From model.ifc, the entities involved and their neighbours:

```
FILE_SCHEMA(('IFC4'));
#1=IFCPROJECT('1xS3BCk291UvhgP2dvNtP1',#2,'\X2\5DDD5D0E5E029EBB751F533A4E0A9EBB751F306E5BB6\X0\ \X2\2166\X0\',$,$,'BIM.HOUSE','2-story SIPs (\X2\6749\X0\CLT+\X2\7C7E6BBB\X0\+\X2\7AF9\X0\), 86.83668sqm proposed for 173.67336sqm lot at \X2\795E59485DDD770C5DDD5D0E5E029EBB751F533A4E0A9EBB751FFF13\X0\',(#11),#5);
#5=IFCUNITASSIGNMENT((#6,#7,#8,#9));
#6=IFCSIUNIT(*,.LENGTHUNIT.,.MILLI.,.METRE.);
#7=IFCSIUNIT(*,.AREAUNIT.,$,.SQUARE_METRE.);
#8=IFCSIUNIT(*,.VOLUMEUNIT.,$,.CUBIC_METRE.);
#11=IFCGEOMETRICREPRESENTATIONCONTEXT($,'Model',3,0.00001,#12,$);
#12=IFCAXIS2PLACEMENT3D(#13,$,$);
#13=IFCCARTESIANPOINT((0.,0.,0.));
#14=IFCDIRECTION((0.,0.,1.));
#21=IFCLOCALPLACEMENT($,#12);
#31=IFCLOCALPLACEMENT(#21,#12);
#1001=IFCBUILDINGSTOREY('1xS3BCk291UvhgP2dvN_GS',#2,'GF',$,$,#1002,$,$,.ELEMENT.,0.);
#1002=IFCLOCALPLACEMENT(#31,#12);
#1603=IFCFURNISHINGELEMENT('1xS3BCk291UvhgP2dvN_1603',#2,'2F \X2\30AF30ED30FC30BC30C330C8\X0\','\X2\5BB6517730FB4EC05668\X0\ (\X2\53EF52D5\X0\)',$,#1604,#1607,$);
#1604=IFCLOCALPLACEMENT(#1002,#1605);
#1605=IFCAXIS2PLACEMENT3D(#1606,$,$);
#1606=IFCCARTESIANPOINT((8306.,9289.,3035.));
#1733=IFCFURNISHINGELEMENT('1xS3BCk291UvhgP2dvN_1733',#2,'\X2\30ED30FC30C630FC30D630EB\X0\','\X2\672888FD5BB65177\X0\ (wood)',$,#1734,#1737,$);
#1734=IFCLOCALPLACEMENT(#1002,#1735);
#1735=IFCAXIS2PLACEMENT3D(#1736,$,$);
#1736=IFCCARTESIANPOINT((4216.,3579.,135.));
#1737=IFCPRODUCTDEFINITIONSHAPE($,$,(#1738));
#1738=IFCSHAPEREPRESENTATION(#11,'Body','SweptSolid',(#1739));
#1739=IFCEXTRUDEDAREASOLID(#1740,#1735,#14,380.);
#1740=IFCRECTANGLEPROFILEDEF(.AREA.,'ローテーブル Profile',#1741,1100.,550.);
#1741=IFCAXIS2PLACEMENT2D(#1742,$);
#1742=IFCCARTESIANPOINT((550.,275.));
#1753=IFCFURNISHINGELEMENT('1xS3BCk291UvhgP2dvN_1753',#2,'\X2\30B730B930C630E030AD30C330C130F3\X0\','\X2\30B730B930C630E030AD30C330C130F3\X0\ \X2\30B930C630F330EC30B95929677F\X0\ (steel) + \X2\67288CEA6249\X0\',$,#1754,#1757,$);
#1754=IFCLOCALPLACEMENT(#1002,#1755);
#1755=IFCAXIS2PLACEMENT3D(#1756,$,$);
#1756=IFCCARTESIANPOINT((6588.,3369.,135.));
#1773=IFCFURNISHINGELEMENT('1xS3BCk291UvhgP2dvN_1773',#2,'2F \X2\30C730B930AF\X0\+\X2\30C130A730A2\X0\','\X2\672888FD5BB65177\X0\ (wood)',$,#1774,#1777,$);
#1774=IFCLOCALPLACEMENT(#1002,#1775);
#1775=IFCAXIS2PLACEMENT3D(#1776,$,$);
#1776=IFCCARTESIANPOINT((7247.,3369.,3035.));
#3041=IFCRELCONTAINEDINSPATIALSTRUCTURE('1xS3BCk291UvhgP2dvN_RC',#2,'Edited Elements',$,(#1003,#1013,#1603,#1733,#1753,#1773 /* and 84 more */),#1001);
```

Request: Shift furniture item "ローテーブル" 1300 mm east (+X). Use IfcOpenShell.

```python
import ifcopenshell
import ifcopenshell.api.geometry
import ifcopenshell.util.placement

model = ifcopenshell.open("model.ifc")

item = model.by_guid("1xS3BCk291UvhgP2dvN_1733")
matrix = ifcopenshell.util.placement.get_local_placement(item.ObjectPlacement)
matrix[0, 3] += 1300.0
ifcopenshell.api.geometry.edit_object_placement(model, product=item, matrix=matrix, is_si=False)

print(ifcopenshell.util.placement.get_local_placement(item.ObjectPlacement).round(3) + 0.0)

model.write("model_edited.ifc")
```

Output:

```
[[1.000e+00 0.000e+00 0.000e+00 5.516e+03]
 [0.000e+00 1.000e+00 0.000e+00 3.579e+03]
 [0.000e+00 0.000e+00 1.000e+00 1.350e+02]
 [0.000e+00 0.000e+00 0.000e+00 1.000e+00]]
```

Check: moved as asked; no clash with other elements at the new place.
